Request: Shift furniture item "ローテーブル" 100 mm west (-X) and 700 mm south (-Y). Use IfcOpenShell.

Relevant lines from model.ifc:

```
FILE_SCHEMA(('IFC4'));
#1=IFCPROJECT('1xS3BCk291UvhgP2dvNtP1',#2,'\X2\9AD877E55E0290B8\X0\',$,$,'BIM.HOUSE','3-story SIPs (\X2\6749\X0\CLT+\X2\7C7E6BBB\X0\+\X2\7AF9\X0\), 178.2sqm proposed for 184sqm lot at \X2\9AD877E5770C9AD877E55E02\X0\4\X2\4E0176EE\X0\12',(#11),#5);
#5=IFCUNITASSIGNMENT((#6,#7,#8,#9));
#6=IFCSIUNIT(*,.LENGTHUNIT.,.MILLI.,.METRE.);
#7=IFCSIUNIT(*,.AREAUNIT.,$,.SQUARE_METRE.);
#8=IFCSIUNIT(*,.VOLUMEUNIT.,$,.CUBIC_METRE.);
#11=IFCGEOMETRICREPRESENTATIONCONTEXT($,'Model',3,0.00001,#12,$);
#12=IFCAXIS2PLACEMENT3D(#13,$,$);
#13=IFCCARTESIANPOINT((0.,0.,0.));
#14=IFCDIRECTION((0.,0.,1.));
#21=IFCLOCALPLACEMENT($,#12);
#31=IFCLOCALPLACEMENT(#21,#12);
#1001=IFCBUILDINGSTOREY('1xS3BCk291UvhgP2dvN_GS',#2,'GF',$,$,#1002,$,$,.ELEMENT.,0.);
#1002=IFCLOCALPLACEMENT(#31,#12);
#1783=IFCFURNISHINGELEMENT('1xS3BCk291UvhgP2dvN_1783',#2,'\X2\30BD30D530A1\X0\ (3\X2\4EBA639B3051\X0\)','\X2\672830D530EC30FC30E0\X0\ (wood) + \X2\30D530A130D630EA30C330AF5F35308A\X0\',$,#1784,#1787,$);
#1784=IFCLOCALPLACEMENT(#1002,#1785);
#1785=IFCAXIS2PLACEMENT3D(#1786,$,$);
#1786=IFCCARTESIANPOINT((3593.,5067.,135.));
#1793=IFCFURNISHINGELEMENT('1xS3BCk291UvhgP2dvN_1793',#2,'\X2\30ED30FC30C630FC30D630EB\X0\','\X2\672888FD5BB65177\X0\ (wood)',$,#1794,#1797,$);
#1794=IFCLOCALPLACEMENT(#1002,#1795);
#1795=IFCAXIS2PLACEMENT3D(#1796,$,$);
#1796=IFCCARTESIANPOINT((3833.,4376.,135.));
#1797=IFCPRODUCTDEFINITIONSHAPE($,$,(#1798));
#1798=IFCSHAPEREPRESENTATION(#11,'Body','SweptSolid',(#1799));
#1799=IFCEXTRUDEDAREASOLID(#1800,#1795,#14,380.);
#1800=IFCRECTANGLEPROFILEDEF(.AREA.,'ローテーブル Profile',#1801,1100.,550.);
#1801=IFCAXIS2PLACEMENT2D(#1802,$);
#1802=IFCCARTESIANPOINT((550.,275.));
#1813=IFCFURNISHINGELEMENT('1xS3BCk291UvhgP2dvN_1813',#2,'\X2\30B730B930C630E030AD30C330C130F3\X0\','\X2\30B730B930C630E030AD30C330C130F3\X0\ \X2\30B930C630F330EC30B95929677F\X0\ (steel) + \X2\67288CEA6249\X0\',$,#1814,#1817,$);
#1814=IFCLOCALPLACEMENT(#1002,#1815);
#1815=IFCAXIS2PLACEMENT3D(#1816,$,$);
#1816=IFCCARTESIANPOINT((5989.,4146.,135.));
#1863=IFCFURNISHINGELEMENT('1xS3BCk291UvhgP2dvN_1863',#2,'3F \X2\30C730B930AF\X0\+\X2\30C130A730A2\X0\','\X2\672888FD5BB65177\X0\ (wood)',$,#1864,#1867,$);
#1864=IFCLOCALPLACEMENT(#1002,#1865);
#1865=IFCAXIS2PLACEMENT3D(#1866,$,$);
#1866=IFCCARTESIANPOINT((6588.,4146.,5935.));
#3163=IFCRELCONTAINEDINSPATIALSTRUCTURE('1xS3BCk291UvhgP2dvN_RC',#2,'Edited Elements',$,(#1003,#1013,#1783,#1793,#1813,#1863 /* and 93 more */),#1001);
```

```python
import ifcopenshell
import ifcopenshell.api.geometry
import ifcopenshell.util.placement
import ifcopenshell.util.unit

model = ifcopenshell.open("model.ifc")
unit_scale = ifcopenshell.util.unit.calculate_unit_scale(model)

item = model.by_guid("1xS3BCk291UvhgP2dvN_1793")
matrix = ifcopenshell.util.placement.get_local_placement(item.ObjectPlacement)
matrix[0, 3] -= 0.1 / unit_scale
matrix[1, 3] -= 0.7 / unit_scale
ifcopenshell.api.geometry.edit_object_placement(model, product=item, matrix=matrix, is_si=False)

print(ifcopenshell.util.placement.get_local_placement(item.ObjectPlacement).round(3) + 0.0)

model.write("model_edited.ifc")
```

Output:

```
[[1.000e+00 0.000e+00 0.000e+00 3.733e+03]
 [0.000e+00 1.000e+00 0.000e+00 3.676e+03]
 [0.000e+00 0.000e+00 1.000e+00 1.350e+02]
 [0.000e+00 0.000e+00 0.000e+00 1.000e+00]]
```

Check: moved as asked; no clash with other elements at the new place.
